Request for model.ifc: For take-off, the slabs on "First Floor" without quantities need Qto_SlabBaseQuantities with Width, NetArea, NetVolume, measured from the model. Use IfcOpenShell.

First a look at what the model holds.

```python
import ifcopenshell
import ifcopenshell.util.element
import ifcopenshell.util.unit

model = ifcopenshell.open("model.ifc")
print(model.schema)
for unit_type in ("LENGTHUNIT", "AREAUNIT", "VOLUMEUNIT"):
    print(unit_type, ifcopenshell.util.unit.calculate_unit_scale(model, unit_type))
storey = next(s for s in model.by_type("IfcBuildingStorey") if s.Name == "First Floor")
slabs = [e for e in ifcopenshell.util.element.get_decomposition(storey) if e.is_a("IfcSlab")]
for e in sorted(slabs, key=lambda e: e.id()):
    print(e.id(), e.is_a(), e.Name, list(ifcopenshell.util.element.get_psets(e, qtos_only=True)), sep=" | ")
```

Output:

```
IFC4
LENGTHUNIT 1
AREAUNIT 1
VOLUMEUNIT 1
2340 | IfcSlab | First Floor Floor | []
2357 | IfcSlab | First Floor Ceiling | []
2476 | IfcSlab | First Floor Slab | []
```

```python
import ifcopenshell
import ifcopenshell.api.pset
import ifcopenshell.geom
import ifcopenshell.util.element
import ifcopenshell.util.shape
import ifcopenshell.util.unit

model = ifcopenshell.open("model.ifc")
unit_scale = ifcopenshell.util.unit.calculate_unit_scale(model)
area_scale = ifcopenshell.util.unit.calculate_unit_scale(model, "AREAUNIT")
volume_scale = ifcopenshell.util.unit.calculate_unit_scale(model, "VOLUMEUNIT")
settings = ifcopenshell.geom.settings()

storey = next(s for s in model.by_type("IfcBuildingStorey") if s.Name == "First Floor")
slabs = [e for e in ifcopenshell.util.element.get_decomposition(storey) if e.is_a("IfcSlab")]

for e in sorted(slabs, key=lambda e: e.id()):
    if ifcopenshell.util.element.get_psets(e, qtos_only=True, should_inherit=False):
        continue
    # Geometry comes back in metres, in the element's own axes.
    shape = ifcopenshell.geom.create_shape(settings, e)
    values = {
        "Width": ifcopenshell.util.shape.get_z(shape.geometry) / unit_scale,
        "NetArea": ifcopenshell.util.shape.get_footprint_area(shape.geometry) / area_scale,
        "NetVolume": ifcopenshell.util.shape.get_volume(shape.geometry) / volume_scale,
    }
    qto = ifcopenshell.api.pset.add_qto(model, product=e, name="Qto_SlabBaseQuantities")
    ifcopenshell.api.pset.edit_qto(model, qto=qto, properties=values)
    print(e.id(), {k: round(v, 3) for k, v in values.items()})

model.write("model_edited.ifc")
```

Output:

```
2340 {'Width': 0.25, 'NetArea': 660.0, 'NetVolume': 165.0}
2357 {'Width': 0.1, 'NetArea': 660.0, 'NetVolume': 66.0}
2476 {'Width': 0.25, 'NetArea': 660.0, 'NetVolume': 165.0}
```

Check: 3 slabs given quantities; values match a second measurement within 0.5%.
